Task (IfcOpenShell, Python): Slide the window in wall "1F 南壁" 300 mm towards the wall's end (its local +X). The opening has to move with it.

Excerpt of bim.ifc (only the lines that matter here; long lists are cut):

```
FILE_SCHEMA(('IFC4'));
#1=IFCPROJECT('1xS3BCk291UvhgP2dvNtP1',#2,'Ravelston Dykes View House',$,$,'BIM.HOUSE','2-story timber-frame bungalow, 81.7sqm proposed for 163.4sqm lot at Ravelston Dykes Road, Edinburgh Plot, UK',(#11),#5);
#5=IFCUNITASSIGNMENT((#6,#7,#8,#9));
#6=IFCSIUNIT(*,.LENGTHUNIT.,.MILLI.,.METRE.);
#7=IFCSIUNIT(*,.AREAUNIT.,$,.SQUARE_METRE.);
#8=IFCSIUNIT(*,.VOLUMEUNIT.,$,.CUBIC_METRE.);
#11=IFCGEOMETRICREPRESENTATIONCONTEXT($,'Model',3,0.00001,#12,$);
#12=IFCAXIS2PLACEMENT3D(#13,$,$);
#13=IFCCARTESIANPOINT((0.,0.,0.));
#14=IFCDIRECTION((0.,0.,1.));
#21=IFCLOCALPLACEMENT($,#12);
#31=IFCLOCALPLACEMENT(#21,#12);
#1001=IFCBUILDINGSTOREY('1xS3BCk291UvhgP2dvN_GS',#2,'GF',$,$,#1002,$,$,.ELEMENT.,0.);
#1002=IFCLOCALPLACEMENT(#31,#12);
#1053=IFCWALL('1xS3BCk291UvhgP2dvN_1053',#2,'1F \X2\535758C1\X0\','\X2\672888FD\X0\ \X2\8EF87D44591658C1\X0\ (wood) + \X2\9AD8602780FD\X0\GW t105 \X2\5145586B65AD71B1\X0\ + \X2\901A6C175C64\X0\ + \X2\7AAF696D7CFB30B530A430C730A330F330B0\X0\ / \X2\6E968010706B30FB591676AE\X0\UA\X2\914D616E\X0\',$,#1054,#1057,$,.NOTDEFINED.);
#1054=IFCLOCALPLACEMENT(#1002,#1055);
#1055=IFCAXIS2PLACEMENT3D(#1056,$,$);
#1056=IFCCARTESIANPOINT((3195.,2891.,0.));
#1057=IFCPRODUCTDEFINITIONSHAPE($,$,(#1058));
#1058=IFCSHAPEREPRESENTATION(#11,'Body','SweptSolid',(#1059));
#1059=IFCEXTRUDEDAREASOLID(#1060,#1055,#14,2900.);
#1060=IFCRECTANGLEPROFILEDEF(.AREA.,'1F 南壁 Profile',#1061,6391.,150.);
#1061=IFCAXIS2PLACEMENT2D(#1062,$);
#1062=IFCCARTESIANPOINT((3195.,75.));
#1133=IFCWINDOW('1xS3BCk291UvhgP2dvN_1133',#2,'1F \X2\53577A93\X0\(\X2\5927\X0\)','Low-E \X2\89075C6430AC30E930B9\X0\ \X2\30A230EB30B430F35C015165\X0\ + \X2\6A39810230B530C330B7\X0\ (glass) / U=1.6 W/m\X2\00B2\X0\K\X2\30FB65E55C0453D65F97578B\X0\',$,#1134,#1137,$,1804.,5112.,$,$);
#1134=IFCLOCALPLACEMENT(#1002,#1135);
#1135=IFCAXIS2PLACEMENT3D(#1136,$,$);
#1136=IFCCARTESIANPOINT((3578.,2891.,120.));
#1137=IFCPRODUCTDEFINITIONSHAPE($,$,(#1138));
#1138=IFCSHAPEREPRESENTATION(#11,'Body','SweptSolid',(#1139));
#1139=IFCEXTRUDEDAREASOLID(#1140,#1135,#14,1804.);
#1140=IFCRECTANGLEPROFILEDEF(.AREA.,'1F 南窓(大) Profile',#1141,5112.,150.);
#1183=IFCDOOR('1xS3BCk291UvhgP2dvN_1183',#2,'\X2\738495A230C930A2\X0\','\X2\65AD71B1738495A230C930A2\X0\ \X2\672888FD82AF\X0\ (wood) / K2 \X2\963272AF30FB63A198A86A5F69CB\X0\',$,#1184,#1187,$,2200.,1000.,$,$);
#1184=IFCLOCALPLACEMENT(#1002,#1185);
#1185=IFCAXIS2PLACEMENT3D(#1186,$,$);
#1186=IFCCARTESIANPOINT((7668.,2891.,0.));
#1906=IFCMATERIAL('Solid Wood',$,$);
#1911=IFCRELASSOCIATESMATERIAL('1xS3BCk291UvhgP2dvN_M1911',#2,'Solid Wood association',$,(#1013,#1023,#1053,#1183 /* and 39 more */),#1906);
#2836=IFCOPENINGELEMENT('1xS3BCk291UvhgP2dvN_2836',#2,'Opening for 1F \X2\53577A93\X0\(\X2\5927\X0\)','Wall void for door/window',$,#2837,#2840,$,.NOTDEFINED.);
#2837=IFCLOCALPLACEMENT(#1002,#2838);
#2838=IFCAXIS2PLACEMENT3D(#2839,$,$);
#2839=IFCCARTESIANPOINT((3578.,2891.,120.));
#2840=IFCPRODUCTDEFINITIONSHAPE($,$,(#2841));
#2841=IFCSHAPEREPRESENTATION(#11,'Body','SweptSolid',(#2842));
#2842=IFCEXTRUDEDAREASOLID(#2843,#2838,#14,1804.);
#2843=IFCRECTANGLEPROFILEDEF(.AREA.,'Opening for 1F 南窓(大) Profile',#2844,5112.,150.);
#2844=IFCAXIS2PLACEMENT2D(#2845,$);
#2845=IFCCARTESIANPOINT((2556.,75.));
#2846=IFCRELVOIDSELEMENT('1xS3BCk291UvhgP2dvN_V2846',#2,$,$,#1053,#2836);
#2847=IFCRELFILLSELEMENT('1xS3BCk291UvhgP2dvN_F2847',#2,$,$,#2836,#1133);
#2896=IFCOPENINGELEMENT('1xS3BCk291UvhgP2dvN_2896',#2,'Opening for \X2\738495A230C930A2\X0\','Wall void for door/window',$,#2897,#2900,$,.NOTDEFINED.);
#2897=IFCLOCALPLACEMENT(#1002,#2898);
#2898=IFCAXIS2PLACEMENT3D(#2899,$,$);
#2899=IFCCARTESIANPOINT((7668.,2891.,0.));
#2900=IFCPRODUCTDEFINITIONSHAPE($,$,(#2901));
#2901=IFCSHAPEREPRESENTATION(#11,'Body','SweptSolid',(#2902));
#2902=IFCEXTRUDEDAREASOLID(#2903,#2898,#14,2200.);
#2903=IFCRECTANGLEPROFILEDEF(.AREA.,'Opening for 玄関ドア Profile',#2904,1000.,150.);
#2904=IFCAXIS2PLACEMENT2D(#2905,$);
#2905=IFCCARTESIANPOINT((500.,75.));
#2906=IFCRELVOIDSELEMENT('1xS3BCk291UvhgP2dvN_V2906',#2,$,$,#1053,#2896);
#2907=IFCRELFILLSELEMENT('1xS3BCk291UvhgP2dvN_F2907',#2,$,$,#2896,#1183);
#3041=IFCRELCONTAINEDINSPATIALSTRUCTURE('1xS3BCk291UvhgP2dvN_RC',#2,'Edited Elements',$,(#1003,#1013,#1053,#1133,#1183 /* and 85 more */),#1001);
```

```python
import ifcopenshell
import ifcopenshell.api.geometry
import ifcopenshell.util.placement
import ifcopenshell.util.unit

model = ifcopenshell.open("bim.ifc")
unit_scale = ifcopenshell.util.unit.calculate_unit_scale(model)

window = model.by_guid("1xS3BCk291UvhgP2dvN_1133")
opening = window.FillsVoids[0].RelatingOpeningElement
wall = opening.VoidsElements[0].RelatingBuildingElement

wall_matrix = ifcopenshell.util.placement.get_local_placement(wall.ObjectPlacement)
shift = wall_matrix[:3, 0] * 0.3 / unit_scale
before = ifcopenshell.util.placement.get_local_placement(window.ObjectPlacement)[:3, 3].copy()

# The window is not placed relative to its opening, so move both.
for product in (opening, window):
    matrix = ifcopenshell.util.placement.get_local_placement(product.ObjectPlacement)
    matrix[:3, 3] += shift
    ifcopenshell.api.geometry.edit_object_placement(model, product=product, matrix=matrix, is_si=False)

after = ifcopenshell.util.placement.get_local_placement(window.ObjectPlacement)[:3, 3]
print("window moved by", (after - before).round(3) + 0.0)

model.write("bim_updated.ifc")
```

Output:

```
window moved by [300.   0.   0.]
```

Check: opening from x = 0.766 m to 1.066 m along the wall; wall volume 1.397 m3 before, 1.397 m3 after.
